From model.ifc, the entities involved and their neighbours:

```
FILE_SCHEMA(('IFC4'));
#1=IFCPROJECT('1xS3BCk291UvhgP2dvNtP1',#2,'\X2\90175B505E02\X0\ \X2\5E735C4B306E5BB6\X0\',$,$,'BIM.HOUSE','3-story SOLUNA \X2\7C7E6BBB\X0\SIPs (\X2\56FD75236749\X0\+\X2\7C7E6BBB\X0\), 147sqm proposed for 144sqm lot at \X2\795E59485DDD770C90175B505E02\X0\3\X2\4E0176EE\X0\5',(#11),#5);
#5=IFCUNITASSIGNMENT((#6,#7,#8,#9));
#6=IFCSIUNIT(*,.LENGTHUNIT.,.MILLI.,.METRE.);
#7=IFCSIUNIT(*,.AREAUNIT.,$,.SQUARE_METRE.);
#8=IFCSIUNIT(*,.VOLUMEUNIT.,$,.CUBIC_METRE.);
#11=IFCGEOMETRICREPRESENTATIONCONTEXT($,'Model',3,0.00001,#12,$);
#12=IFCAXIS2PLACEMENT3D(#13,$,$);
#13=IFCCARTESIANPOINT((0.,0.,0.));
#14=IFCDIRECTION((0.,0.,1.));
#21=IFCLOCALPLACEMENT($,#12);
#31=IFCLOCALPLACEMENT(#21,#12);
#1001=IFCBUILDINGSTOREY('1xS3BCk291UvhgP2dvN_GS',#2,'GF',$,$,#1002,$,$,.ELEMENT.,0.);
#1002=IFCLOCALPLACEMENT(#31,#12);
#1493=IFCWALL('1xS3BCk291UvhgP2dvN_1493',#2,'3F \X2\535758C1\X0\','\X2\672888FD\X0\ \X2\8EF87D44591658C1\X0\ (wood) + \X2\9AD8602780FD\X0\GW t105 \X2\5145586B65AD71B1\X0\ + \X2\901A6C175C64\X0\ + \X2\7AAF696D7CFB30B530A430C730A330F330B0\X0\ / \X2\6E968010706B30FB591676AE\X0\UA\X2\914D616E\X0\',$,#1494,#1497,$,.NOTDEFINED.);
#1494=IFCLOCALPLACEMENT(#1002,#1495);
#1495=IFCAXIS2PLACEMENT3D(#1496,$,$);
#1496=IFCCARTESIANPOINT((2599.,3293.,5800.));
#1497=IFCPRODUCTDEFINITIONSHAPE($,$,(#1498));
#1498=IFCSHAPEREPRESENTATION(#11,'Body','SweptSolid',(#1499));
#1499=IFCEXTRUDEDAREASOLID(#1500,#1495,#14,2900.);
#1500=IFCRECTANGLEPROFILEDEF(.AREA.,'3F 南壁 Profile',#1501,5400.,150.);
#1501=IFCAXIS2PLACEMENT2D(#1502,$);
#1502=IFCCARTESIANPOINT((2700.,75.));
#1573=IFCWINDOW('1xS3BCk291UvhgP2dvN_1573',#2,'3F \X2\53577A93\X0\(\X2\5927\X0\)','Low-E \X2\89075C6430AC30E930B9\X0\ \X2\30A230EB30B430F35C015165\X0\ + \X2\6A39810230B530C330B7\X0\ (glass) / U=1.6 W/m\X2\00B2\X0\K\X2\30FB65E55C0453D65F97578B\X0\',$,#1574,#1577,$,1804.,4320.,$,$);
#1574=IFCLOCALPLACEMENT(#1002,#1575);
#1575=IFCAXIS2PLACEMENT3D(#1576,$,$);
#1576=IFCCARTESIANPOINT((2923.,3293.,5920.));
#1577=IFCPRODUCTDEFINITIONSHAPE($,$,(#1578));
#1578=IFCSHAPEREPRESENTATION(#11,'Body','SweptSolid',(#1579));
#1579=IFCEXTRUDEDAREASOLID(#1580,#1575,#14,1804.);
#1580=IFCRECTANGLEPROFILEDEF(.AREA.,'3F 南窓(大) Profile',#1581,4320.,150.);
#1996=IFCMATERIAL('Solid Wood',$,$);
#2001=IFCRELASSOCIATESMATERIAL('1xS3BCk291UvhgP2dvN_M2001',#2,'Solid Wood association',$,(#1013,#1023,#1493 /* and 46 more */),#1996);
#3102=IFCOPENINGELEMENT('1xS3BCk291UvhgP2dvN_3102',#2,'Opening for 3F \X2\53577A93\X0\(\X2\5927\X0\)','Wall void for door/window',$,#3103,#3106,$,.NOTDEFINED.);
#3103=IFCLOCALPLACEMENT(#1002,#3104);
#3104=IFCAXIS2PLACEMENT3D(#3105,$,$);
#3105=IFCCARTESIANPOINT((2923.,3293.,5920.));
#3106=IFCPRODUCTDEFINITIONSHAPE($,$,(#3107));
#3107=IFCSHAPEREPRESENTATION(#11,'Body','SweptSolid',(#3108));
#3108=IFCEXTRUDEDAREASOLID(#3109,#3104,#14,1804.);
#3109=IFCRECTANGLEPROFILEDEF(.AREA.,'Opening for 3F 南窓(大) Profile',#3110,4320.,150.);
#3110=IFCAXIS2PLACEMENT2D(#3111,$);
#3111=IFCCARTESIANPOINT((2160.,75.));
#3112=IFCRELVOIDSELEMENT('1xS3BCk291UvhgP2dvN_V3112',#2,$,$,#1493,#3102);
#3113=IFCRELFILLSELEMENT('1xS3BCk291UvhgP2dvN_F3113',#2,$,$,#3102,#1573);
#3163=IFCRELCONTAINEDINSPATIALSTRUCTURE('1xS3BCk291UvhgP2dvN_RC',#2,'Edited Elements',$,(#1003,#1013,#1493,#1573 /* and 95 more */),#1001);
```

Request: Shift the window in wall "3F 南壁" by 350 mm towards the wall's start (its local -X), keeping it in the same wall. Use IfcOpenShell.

```python
import ifcopenshell
import ifcopenshell.api.geometry
import ifcopenshell.util.placement

model = ifcopenshell.open("model.ifc")

window = model.by_id(1573)
opening = window.FillsVoids[0].RelatingOpeningElement
wall = opening.VoidsElements[0].RelatingBuildingElement

wall_matrix = ifcopenshell.util.placement.get_local_placement(wall.ObjectPlacement)
shift = wall_matrix[:3, 0] * -350.0
before = ifcopenshell.util.placement.get_local_placement(window.ObjectPlacement)[:3, 3].copy()

# The window is not placed relative to its opening, so move both.
for product in (opening, window):
    matrix = ifcopenshell.util.placement.get_local_placement(product.ObjectPlacement)
    matrix[:3, 3] += shift
    ifcopenshell.api.geometry.edit_object_placement(model, product=product, matrix=matrix, is_si=False)

after = ifcopenshell.util.placement.get_local_placement(window.ObjectPlacement)[:3, 3]
print("window moved by", (after - before).round(3) + 0.0)

model.write("model_v2.ifc")
```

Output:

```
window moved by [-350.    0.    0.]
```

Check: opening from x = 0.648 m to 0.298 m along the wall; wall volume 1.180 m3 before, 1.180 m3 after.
